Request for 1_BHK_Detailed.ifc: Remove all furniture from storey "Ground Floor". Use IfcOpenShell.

First a look at what the model holds.

```python
import ifcopenshell
import ifcopenshell.util.element

model = ifcopenshell.open("1_BHK_Detailed.ifc")
print(model.schema)
storey = next(s for s in model.by_type("IfcBuildingStorey") if s.Name == "Ground Floor")
furniture = [e for e in ifcopenshell.util.element.get_decomposition(storey) if e.is_a("IfcFurnishingElement")]
seen = {}
for e in furniture:
    element_type = ifcopenshell.util.element.get_type(e)
    name = element_type.Name if element_type not in (None, e) else None
    seen[name] = seen.get(name, 0) + 1
for name, count in sorted(seen.items(), key=str):
    print(count, "x", name)
```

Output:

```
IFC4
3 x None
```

```python
import ifcopenshell
import ifcopenshell.api.root
import ifcopenshell.util.element

model = ifcopenshell.open("1_BHK_Detailed.ifc")

storey = next(s for s in model.by_type("IfcBuildingStorey") if s.Name == "Ground Floor")
furniture = [e for e in ifcopenshell.util.element.get_decomposition(storey) if e.is_a("IfcFurnishingElement")]

for e in furniture:
    ifcopenshell.api.root.remove_product(model, product=e)
print(len(furniture), "removed")

model.write("1_BHK_Detailed_updated.ifc")
```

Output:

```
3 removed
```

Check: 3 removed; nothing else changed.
